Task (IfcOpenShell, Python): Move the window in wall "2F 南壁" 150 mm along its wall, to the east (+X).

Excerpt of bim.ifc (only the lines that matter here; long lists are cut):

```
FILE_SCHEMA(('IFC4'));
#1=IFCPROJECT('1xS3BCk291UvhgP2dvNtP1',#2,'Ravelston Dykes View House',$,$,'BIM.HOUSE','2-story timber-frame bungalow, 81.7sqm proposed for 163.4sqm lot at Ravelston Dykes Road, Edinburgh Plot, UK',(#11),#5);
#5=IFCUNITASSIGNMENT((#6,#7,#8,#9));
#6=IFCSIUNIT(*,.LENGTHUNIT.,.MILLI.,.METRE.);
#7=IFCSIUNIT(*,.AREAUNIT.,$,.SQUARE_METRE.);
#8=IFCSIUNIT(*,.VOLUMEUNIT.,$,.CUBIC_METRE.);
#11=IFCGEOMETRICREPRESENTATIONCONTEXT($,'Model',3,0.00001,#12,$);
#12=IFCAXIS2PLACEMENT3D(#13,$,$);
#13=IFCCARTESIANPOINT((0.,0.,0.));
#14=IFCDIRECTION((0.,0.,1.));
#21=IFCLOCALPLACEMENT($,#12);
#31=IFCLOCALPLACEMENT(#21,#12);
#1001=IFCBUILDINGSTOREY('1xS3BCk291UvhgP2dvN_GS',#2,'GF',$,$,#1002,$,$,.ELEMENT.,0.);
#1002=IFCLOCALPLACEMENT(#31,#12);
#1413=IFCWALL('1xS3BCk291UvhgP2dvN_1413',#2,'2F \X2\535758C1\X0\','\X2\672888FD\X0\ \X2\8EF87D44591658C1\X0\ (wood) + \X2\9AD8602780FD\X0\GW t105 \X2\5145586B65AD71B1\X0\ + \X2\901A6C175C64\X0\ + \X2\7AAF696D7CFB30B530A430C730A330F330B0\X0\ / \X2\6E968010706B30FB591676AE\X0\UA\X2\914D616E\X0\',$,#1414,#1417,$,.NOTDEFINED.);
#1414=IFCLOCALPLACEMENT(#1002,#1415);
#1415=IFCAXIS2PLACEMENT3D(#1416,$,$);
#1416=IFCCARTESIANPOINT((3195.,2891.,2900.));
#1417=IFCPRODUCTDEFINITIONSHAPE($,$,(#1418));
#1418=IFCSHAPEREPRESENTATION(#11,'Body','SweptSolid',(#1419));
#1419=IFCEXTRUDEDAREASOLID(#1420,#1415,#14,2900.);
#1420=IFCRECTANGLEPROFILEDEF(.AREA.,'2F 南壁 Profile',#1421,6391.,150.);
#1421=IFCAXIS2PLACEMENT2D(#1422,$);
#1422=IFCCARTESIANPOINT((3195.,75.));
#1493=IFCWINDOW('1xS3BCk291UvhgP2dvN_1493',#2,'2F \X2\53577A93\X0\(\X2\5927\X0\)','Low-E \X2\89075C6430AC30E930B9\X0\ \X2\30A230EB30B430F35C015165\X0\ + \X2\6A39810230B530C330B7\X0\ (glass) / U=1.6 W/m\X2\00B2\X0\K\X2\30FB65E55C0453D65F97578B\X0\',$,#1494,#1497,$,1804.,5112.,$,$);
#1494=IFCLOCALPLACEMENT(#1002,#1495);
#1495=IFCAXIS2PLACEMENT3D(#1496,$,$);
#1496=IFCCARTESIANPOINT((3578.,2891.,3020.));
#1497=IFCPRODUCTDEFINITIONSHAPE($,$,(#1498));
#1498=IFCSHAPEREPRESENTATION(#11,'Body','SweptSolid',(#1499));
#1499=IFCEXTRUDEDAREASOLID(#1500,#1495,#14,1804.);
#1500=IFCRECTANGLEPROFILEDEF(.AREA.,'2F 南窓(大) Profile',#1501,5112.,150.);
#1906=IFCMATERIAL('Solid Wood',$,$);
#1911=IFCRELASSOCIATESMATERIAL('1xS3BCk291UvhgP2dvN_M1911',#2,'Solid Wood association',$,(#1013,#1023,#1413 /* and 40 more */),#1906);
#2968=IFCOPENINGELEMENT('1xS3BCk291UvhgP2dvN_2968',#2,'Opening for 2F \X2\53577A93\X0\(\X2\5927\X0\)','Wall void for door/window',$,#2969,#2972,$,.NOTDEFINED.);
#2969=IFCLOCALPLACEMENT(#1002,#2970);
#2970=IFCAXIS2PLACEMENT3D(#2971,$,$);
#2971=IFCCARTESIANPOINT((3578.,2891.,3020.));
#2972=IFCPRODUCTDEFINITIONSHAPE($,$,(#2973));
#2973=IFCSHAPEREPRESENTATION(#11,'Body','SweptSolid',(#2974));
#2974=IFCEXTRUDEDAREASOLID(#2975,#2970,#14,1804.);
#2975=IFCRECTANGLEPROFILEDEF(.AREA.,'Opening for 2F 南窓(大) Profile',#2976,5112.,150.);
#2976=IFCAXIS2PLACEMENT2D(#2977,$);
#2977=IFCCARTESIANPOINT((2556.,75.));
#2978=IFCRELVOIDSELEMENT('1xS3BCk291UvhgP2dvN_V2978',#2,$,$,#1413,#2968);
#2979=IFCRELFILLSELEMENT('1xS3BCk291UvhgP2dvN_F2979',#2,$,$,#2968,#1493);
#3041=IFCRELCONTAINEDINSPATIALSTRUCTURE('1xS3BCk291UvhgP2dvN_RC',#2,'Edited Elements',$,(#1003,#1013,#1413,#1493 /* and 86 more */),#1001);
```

```python
import ifcopenshell
import ifcopenshell.api.geometry
import ifcopenshell.util.placement
import ifcopenshell.util.unit

model = ifcopenshell.open("bim.ifc")
unit_scale = ifcopenshell.util.unit.calculate_unit_scale(model)

window = model.by_id(1493)
opening = window.FillsVoids[0].RelatingOpeningElement
wall = opening.VoidsElements[0].RelatingBuildingElement

wall_matrix = ifcopenshell.util.placement.get_local_placement(wall.ObjectPlacement)
shift = wall_matrix[:3, 0] * 0.15 / unit_scale
before = ifcopenshell.util.placement.get_local_placement(window.ObjectPlacement)[:3, 3].copy()

# The window is not placed relative to its opening, so move both.
for product in (opening, window):
    matrix = ifcopenshell.util.placement.get_local_placement(product.ObjectPlacement)
    matrix[:3, 3] += shift
    ifcopenshell.api.geometry.edit_object_placement(model, product=product, matrix=matrix, is_si=False)

after = ifcopenshell.util.placement.get_local_placement(window.ObjectPlacement)[:3, 3]
print("window moved by", (after - before).round(3) + 0.0)

model.write("bim_edited.ifc")
```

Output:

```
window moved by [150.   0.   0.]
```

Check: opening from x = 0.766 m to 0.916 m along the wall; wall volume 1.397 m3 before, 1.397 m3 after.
